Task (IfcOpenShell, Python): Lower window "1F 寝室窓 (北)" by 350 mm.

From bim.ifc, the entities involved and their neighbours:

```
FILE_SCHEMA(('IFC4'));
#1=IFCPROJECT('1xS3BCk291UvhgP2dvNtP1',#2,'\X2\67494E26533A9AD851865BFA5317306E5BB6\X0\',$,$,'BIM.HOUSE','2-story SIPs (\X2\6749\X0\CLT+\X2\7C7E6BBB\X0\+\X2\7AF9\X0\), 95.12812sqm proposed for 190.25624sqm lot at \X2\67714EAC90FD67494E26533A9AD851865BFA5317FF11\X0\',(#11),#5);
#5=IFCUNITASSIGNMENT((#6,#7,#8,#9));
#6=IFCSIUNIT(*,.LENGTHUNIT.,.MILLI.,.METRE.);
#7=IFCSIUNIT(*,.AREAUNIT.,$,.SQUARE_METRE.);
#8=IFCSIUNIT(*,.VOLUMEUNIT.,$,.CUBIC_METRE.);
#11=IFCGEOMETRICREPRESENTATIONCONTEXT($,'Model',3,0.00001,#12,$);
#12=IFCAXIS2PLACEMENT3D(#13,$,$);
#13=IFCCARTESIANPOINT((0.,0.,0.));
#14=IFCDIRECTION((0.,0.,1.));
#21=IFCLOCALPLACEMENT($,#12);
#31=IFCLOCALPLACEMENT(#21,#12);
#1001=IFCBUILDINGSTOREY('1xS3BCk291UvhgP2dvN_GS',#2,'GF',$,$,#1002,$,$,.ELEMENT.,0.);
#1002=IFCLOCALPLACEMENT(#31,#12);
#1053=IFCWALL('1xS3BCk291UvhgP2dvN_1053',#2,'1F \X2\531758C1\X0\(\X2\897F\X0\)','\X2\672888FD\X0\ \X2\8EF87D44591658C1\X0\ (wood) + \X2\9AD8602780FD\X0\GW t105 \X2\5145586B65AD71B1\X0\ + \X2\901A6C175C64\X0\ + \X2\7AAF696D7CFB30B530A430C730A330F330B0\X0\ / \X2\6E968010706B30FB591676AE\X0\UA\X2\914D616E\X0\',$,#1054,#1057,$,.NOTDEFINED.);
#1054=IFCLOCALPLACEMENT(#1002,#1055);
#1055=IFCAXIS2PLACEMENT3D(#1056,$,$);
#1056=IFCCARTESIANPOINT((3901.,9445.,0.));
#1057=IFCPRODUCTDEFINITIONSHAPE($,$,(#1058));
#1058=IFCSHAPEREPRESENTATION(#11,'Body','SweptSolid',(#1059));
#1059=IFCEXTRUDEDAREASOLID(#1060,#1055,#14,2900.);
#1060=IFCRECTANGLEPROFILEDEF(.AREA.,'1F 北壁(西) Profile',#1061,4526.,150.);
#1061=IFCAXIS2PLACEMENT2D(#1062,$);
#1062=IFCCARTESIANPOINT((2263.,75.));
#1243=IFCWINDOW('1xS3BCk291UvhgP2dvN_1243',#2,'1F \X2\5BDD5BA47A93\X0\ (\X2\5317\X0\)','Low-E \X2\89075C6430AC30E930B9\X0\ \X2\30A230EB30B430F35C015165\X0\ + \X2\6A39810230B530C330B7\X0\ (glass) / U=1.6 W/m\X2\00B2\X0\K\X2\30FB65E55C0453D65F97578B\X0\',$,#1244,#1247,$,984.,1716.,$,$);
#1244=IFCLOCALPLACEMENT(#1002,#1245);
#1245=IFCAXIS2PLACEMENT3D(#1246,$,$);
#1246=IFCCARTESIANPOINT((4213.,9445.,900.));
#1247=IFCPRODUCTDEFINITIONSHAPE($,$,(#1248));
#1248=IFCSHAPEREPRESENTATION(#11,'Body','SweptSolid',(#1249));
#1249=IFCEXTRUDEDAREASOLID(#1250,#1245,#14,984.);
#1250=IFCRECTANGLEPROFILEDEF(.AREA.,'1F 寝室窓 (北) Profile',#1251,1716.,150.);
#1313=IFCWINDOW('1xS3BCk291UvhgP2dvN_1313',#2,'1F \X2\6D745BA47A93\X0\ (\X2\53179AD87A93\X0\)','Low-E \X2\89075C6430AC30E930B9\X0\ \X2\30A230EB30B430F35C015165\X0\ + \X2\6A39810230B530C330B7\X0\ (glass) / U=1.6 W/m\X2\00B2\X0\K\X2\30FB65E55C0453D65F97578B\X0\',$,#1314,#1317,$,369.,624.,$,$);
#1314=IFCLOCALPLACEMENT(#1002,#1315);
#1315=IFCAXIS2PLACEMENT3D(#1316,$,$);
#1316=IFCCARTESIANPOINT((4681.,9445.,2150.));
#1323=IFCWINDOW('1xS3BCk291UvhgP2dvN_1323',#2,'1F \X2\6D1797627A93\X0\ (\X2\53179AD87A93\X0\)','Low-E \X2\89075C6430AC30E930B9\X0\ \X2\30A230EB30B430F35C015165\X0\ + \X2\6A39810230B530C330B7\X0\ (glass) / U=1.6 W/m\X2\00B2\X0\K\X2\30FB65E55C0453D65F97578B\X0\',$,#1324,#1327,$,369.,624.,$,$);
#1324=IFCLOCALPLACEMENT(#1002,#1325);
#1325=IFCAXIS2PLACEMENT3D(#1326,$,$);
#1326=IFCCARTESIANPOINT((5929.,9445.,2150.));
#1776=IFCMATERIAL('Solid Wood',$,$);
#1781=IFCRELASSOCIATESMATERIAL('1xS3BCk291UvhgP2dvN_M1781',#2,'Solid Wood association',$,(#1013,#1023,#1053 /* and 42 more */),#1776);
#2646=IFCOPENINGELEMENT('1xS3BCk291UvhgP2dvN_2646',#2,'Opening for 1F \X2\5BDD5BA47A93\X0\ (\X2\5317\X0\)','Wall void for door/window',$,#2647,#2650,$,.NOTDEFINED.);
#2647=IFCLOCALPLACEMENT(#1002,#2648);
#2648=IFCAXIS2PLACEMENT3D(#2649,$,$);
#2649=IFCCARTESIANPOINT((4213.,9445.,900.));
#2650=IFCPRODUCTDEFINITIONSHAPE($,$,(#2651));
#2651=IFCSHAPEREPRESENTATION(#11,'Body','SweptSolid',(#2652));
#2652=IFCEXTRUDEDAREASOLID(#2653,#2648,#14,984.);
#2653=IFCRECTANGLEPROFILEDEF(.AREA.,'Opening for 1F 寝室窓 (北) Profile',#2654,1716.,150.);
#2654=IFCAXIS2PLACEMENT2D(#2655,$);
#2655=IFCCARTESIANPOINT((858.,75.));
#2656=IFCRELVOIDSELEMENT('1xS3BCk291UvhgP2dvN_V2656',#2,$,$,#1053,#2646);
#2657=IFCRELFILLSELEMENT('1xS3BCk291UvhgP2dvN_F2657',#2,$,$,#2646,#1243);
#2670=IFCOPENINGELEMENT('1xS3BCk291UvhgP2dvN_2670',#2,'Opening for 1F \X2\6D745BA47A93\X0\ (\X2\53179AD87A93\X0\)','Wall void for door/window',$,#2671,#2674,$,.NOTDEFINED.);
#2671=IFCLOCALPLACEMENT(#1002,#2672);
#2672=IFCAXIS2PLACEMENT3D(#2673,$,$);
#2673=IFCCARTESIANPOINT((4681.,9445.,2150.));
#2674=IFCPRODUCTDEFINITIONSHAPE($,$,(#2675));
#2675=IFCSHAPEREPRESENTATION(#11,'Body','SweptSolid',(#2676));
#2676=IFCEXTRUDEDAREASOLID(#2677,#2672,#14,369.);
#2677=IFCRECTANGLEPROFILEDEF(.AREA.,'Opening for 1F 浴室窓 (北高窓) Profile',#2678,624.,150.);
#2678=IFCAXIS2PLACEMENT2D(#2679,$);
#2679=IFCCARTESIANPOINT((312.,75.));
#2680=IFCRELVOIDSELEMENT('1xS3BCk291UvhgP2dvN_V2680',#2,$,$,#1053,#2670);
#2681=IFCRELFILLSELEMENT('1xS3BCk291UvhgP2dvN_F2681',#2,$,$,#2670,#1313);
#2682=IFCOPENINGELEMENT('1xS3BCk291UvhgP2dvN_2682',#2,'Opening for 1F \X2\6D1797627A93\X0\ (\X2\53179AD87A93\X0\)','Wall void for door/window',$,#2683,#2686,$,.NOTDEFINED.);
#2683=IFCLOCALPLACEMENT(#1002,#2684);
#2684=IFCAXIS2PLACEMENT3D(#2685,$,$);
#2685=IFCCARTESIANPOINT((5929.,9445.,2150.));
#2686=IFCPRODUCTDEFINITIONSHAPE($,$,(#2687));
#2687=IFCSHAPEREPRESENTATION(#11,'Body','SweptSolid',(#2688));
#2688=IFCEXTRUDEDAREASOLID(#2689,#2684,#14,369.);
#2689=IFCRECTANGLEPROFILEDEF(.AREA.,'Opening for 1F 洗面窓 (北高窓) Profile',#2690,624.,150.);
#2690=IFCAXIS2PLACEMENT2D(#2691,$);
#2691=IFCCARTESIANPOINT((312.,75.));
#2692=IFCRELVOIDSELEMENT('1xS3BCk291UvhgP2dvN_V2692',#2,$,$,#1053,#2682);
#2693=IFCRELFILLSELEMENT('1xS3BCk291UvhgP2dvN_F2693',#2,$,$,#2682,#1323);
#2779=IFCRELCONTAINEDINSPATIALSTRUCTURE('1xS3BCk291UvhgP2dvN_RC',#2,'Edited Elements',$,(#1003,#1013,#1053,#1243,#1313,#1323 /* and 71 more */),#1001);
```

```python
import numpy as np
import ifcopenshell
import ifcopenshell.api.geometry
import ifcopenshell.util.placement
import ifcopenshell.util.unit

model = ifcopenshell.open("bim.ifc")
unit_scale = ifcopenshell.util.unit.calculate_unit_scale(model)

window = model.by_guid("1xS3BCk291UvhgP2dvN_1243")
opening = window.FillsVoids[0].RelatingOpeningElement
dz = -0.35 / unit_scale

shift = np.array([0.0, 0.0, dz])
# The window is not placed relative to its opening, so move both.
for product in (opening, window):
    matrix = ifcopenshell.util.placement.get_local_placement(product.ObjectPlacement)
    matrix[:3, 3] += shift
    ifcopenshell.api.geometry.edit_object_placement(model, product=product, matrix=matrix, is_si=False)

print(f"moved by {dz * unit_scale:+.3f} m")

model.write("bim_rev.ifc")
```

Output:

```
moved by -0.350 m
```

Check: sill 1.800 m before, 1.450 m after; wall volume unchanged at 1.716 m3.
